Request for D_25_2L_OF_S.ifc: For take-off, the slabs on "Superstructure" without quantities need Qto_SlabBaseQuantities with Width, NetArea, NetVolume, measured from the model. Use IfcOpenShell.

First a look at what the model holds.

```python
import ifcopenshell
import ifcopenshell.util.element
import ifcopenshell.util.unit

model = ifcopenshell.open("D_25_2L_OF_S.ifc")
print(model.schema)
for unit_type in ("LENGTHUNIT", "AREAUNIT", "VOLUMEUNIT"):
    print(unit_type, ifcopenshell.util.unit.calculate_unit_scale(model, unit_type))
storey = next(s for s in model.by_type("IfcBuildingStorey") if s.Name == "Superstructure")
slabs = [e for e in ifcopenshell.util.element.get_decomposition(storey) if e.is_a("IfcSlab")]
for e in sorted(slabs, key=lambda e: e.id()):
    print(e.id(), e.is_a(), e.Name, list(ifcopenshell.util.element.get_psets(e, qtos_only=True)), sep=" | ")
```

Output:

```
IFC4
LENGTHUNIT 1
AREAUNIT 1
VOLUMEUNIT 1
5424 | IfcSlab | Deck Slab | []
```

```python
import ifcopenshell
import ifcopenshell.api.pset
import ifcopenshell.geom
import ifcopenshell.util.element
import ifcopenshell.util.shape
import ifcopenshell.util.unit

model = ifcopenshell.open("D_25_2L_OF_S.ifc")
unit_scale = ifcopenshell.util.unit.calculate_unit_scale(model)
area_scale = ifcopenshell.util.unit.calculate_unit_scale(model, "AREAUNIT")
volume_scale = ifcopenshell.util.unit.calculate_unit_scale(model, "VOLUMEUNIT")
settings = ifcopenshell.geom.settings()

storey = next(s for s in model.by_type("IfcBuildingStorey") if s.Name == "Superstructure")
slabs = [e for e in ifcopenshell.util.element.get_decomposition(storey) if e.is_a("IfcSlab")]

for e in sorted(slabs, key=lambda e: e.id()):
    if ifcopenshell.util.element.get_psets(e, qtos_only=True, should_inherit=False):
        continue
    # Geometry comes back in metres, in the element's own axes.
    shape = ifcopenshell.geom.create_shape(settings, e)
    values = {
        "Width": ifcopenshell.util.shape.get_z(shape.geometry) / unit_scale,
        "NetArea": ifcopenshell.util.shape.get_footprint_area(shape.geometry) / area_scale,
        "NetVolume": ifcopenshell.util.shape.get_volume(shape.geometry) / volume_scale,
    }
    qto = ifcopenshell.api.pset.add_qto(model, product=e, name="Qto_SlabBaseQuantities")
    ifcopenshell.api.pset.edit_qto(model, qto=qto, properties=values)
    print(e.id(), {k: round(v, 3) for k, v in values.items()})

model.write("D_25_2L_OF_S_rev.ifc")
```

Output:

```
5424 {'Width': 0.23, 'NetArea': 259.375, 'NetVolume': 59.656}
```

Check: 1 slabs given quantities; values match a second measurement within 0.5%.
